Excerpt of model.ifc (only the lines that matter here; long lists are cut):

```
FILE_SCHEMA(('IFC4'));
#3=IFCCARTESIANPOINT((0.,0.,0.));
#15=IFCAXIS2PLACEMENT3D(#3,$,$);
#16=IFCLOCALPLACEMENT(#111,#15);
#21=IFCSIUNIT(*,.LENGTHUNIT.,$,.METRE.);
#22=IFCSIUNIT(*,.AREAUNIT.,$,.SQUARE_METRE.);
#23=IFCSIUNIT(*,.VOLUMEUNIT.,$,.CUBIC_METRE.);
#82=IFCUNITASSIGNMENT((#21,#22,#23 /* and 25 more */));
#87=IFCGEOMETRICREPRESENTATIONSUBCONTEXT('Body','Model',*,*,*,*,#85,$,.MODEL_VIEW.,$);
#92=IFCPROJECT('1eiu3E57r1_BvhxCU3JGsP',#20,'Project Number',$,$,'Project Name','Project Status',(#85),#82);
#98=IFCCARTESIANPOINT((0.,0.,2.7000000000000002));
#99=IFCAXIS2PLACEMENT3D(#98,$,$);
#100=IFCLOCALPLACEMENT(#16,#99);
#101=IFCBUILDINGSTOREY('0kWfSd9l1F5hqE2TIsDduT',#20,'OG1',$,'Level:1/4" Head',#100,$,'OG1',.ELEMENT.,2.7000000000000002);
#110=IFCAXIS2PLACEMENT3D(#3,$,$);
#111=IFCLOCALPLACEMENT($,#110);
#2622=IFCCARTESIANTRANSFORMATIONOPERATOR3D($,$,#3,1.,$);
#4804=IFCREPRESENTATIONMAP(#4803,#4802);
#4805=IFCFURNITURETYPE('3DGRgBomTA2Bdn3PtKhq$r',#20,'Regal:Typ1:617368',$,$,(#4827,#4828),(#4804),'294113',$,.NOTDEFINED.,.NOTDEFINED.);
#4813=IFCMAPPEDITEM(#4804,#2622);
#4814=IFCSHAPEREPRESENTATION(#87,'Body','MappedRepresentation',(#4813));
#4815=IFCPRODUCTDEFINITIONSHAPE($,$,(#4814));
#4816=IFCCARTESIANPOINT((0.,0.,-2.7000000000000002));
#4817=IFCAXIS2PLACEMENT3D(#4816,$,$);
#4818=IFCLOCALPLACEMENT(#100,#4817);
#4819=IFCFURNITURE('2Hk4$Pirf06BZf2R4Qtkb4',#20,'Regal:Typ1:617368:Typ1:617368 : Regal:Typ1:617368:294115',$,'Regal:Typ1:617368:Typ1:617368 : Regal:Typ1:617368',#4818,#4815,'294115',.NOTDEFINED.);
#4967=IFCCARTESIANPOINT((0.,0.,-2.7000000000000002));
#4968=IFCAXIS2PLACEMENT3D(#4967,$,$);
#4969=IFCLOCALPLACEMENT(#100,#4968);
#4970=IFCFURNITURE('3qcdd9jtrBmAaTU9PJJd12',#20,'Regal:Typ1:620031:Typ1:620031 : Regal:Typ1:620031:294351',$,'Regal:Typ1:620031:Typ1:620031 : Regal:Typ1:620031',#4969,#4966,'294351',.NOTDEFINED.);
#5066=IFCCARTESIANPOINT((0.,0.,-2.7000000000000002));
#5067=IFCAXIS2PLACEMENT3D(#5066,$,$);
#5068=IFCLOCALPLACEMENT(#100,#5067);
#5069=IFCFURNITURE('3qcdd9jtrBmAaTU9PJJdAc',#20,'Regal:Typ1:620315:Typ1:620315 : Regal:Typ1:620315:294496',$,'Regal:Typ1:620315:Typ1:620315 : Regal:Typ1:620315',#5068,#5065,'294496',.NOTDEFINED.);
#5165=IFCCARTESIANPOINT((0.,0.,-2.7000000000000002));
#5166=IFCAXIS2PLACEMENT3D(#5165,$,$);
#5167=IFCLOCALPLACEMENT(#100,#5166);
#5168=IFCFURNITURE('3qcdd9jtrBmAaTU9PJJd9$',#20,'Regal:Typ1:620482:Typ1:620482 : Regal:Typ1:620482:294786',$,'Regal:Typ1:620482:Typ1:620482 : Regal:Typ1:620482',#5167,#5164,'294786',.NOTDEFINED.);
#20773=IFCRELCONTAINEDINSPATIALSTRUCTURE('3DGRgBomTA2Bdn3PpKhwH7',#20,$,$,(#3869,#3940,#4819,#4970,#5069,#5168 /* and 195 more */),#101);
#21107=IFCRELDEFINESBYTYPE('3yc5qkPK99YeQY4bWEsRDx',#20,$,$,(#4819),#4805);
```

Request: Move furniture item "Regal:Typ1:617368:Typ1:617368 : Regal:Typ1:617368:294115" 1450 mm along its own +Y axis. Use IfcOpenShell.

```python
import ifcopenshell
import ifcopenshell.api.geometry
import ifcopenshell.util.placement

model = ifcopenshell.open("model.ifc")

item = model.by_guid("2Hk4$Pirf06BZf2R4Qtkb4")
matrix = ifcopenshell.util.placement.get_local_placement(item.ObjectPlacement)
matrix[:3, 3] += matrix[:3, 1] * 1.45
ifcopenshell.api.geometry.edit_object_placement(model, product=item, matrix=matrix, is_si=False)

print(ifcopenshell.util.placement.get_local_placement(item.ObjectPlacement).round(3) + 0.0)

model.write("model_edited.ifc")
```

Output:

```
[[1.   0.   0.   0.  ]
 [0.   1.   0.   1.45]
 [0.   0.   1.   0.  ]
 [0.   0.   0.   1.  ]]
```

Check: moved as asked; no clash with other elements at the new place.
